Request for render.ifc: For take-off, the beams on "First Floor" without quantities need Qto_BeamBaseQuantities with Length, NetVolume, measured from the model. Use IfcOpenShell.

First a look at what the model holds.

```python
import ifcopenshell
import ifcopenshell.util.element
import ifcopenshell.util.unit

model = ifcopenshell.open("render.ifc")
print(model.schema)
for unit_type in ("LENGTHUNIT", "AREAUNIT", "VOLUMEUNIT"):
    print(unit_type, ifcopenshell.util.unit.calculate_unit_scale(model, unit_type))
storey = next(s for s in model.by_type("IfcBuildingStorey") if s.Name == "First Floor")
beams = [e for e in ifcopenshell.util.element.get_decomposition(storey) if e.is_a("IfcBeam")]
for e in sorted(beams, key=lambda e: e.id()):
    print(e.id(), e.is_a(), e.Name, list(ifcopenshell.util.element.get_psets(e, qtos_only=True)), sep=" | ")
```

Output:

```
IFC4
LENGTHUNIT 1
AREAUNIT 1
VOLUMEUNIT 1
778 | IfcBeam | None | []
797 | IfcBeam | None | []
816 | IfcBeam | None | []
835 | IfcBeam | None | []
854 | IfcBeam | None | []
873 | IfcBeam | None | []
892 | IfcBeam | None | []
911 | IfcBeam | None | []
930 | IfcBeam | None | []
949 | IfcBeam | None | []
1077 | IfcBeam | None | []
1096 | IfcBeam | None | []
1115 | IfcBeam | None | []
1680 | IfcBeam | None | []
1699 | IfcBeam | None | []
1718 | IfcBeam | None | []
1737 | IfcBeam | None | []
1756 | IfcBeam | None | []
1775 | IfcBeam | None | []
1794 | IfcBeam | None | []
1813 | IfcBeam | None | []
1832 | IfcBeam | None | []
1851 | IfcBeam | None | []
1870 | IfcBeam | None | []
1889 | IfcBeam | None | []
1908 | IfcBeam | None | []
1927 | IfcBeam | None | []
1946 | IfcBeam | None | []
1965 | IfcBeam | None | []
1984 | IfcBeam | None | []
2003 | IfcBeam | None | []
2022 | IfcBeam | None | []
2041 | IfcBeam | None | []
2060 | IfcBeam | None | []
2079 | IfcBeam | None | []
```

```python
import ifcopenshell
import ifcopenshell.api.pset
import ifcopenshell.geom
import ifcopenshell.util.element
import ifcopenshell.util.shape
import ifcopenshell.util.unit

model = ifcopenshell.open("render.ifc")
unit_scale = ifcopenshell.util.unit.calculate_unit_scale(model)
volume_scale = ifcopenshell.util.unit.calculate_unit_scale(model, "VOLUMEUNIT")
settings = ifcopenshell.geom.settings()

storey = next(s for s in model.by_type("IfcBuildingStorey") if s.Name == "First Floor")
beams = [e for e in ifcopenshell.util.element.get_decomposition(storey) if e.is_a("IfcBeam")]

for e in sorted(beams, key=lambda e: e.id()):
    if ifcopenshell.util.element.get_psets(e, qtos_only=True, should_inherit=False):
        continue
    # Geometry comes back in metres, in the element's own axes.
    shape = ifcopenshell.geom.create_shape(settings, e)
    values = {
        "Length": ifcopenshell.util.shape.get_max_xyz(shape.geometry) / unit_scale,
        "NetVolume": ifcopenshell.util.shape.get_volume(shape.geometry) / volume_scale,
    }
    qto = ifcopenshell.api.pset.add_qto(model, product=e, name="Qto_BeamBaseQuantities")
    ifcopenshell.api.pset.edit_qto(model, qto=qto, properties=values)
    print(e.id(), {k: round(v, 3) for k, v in values.items()})

model.write("render_edited.ifc")
```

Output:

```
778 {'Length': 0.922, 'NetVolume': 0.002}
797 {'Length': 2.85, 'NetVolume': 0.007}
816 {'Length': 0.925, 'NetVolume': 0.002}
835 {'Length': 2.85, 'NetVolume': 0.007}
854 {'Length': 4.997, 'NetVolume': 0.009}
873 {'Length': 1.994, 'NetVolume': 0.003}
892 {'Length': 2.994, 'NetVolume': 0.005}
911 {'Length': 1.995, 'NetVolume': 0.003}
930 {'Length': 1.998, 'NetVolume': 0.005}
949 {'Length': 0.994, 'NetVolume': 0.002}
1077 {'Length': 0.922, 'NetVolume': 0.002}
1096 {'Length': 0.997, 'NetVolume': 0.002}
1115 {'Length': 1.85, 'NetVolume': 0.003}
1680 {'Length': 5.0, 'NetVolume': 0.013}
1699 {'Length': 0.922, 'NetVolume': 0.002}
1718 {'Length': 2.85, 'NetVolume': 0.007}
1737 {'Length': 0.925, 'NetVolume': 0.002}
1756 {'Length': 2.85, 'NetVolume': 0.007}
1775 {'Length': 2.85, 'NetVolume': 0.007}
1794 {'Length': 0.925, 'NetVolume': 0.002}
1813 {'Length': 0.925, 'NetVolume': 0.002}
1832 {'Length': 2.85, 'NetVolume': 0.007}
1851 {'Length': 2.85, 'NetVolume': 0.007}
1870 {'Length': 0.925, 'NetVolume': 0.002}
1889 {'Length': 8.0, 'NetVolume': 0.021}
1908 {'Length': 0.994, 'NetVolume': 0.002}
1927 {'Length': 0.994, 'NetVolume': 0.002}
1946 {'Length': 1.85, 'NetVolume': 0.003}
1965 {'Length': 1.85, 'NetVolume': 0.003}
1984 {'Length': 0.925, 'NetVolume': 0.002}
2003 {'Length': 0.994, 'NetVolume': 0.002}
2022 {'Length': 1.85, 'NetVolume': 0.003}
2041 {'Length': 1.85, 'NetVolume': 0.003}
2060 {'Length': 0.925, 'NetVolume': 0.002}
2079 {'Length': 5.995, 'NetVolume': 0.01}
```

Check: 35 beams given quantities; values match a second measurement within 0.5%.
